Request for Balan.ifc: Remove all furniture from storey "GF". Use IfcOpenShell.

First a look at what the model holds.

```python
import ifcopenshell
import ifcopenshell.util.element

model = ifcopenshell.open("Balan.ifc")
print(model.schema)
storey = next(s for s in model.by_type("IfcBuildingStorey") if s.Name == "GF")
furniture = [e for e in ifcopenshell.util.element.get_decomposition(storey) if e.is_a("IfcFurnishingElement")]
seen = {}
for e in furniture:
    element_type = ifcopenshell.util.element.get_type(e)
    name = element_type.Name if element_type not in (None, e) else None
    seen[name] = seen.get(name, 0) + 1
for name, count in sorted(seen.items(), key=str):
    print(count, "x", name)
```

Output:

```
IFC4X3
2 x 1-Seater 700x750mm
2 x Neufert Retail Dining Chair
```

```python
import ifcopenshell
import ifcopenshell.api.root
import ifcopenshell.util.element

model = ifcopenshell.open("Balan.ifc")

storey = next(s for s in model.by_type("IfcBuildingStorey") if s.Name == "GF")
furniture = [e for e in ifcopenshell.util.element.get_decomposition(storey) if e.is_a("IfcFurnishingElement")]

for e in furniture:
    ifcopenshell.api.root.remove_product(model, product=e)
print(len(furniture), "removed")

model.write("Balan-out.ifc")
```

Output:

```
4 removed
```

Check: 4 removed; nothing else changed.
